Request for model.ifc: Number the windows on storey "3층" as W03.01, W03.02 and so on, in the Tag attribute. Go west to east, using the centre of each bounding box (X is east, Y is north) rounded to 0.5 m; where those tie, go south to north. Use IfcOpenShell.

First a look at what the model holds.

```python
import ifcopenshell
import ifcopenshell.util.element
import ifcopenshell.util.placement

model = ifcopenshell.open("model.ifc")
print(model.schema)
storey = next(s for s in model.by_type("IfcBuildingStorey") if s.Name == "3층")
windows = [e for e in ifcopenshell.util.element.get_decomposition(storey) if e.is_a("IfcWindow")]
for e in sorted(windows, key=lambda e: e.id()):
    origin = ifcopenshell.util.placement.get_local_placement(e.ObjectPlacement)[:3, 3]
    print(e.id(), e.Tag, e.Name, origin.round(2) + 0.0, sep=" | ")
```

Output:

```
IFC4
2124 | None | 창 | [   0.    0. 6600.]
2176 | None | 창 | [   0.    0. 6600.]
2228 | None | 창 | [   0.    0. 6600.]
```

```python
import ifcopenshell
import ifcopenshell.geom
import ifcopenshell.util.element
import ifcopenshell.util.shape

model = ifcopenshell.open("model.ifc")
settings = ifcopenshell.geom.settings()
settings.set("use-world-coords", True)


def centre(element):
    shape = ifcopenshell.geom.create_shape(settings, element)
    return ifcopenshell.util.shape.get_bbox_centroid(shape.geometry)


storey = next(s for s in model.by_type("IfcBuildingStorey") if s.Name == "3층")
windows = [e for e in ifcopenshell.util.element.get_decomposition(storey) if e.is_a("IfcWindow")]

# Insertion points can sit at a corner or the storey origin, so sort by the geometry (in metres).
centres = {e: centre(e) for e in windows}
windows.sort(key=lambda e: (round(centres[e][0] / 0.5), centres[e][1]))

for i, e in enumerate(windows, start=1):
    number = f"W03.{i:02d}"
    e.Tag = number
    print(e.id(), number)

model.write("model_v2.ifc")
```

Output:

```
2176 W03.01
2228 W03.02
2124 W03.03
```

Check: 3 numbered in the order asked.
